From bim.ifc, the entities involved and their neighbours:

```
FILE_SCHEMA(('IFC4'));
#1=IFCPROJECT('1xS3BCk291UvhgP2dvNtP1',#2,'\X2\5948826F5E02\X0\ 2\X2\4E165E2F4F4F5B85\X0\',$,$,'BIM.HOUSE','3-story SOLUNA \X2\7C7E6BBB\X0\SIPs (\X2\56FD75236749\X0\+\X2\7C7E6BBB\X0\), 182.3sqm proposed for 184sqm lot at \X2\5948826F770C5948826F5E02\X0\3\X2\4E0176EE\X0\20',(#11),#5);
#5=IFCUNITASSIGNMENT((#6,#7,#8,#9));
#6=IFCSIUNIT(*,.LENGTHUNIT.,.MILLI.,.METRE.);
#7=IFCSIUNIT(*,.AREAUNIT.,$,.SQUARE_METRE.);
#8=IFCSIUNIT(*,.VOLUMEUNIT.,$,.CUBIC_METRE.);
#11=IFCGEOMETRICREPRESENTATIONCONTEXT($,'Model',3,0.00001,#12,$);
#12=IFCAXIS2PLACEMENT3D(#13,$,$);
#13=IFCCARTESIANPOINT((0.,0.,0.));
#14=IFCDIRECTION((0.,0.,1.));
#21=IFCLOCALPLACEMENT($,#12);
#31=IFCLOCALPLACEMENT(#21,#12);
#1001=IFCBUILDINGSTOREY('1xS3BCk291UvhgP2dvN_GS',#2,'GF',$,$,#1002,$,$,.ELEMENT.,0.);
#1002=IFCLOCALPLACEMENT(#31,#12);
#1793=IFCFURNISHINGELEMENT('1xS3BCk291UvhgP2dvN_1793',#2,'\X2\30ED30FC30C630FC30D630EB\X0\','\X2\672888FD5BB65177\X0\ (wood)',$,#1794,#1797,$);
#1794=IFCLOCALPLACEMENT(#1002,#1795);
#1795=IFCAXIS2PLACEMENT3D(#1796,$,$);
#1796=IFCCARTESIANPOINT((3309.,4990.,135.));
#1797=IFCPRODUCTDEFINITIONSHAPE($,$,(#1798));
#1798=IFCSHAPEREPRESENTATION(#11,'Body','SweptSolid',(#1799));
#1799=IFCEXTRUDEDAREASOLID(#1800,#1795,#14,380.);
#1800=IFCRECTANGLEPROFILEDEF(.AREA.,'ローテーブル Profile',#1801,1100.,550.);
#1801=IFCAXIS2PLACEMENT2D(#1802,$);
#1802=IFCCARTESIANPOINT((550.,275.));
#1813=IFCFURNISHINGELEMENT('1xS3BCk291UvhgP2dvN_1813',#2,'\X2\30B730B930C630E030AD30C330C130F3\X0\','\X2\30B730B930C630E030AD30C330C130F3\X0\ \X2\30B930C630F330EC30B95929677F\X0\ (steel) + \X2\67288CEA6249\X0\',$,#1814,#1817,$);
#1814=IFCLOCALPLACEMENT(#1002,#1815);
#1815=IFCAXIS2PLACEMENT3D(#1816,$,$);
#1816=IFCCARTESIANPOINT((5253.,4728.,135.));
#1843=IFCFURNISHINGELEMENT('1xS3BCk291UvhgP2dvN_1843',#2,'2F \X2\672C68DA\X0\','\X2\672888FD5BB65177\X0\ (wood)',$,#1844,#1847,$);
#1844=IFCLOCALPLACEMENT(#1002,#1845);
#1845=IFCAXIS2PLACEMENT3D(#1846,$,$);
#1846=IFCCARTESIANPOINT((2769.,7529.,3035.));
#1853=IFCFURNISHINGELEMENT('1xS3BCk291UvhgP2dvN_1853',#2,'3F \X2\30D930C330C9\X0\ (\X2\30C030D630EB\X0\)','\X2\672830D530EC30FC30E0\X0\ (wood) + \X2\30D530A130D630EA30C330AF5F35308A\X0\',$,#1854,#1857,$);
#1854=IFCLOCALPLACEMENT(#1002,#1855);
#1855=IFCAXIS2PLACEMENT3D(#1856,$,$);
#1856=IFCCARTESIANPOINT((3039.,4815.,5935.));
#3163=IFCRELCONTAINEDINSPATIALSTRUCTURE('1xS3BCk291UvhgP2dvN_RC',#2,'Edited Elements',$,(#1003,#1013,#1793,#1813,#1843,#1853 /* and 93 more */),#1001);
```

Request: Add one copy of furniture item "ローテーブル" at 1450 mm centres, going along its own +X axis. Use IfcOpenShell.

```python
import ifcopenshell
import ifcopenshell.api.geometry
import ifcopenshell.api.root
import ifcopenshell.util.element
import ifcopenshell.util.placement
import ifcopenshell.util.unit

model = ifcopenshell.open("bim.ifc")
unit_scale = ifcopenshell.util.unit.calculate_unit_scale(model)


def reuse_history(source, copy):
    """copy_class also copies each property set's owner history, people and application; keep the originals."""
    for rel in copy.IsDefinedBy:
        if rel.is_a("IfcRelDefinesByProperties") and (history := rel.RelatingPropertyDefinition.OwnerHistory):
            rel.RelatingPropertyDefinition.OwnerHistory = source.OwnerHistory
            ifcopenshell.util.element.remove_deep2(model, history)


source = model.by_id(1793)
base = ifcopenshell.util.placement.get_local_placement(source.ObjectPlacement)
step = base[:3, 0] * 1.45 / unit_scale

for i in range(1, 2):
    copy = ifcopenshell.api.root.copy_class(model, product=source)
    copy.Representation = ifcopenshell.util.element.copy_deep(
        model, source.Representation, exclude=["IfcGeometricRepresentationContext", "IfcRepresentationMap"]
    )
    reuse_history(source, copy)
    matrix = base.copy()
    matrix[:3, 3] += i * step
    print("added at", matrix[:3, 3].round(3) + 0.0)
    ifcopenshell.api.geometry.edit_object_placement(model, product=copy, matrix=matrix, is_si=False)

model.write("bim-out.ifc")
```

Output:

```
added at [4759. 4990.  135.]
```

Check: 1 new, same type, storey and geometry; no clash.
